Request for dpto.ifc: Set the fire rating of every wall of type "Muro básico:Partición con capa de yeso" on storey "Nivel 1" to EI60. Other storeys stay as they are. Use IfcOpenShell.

First a look at what the model holds.

```python
import ifcopenshell
import ifcopenshell.util.element

model = ifcopenshell.open("dpto.ifc")
print(model.schema)
storey = next(s for s in model.by_type("IfcBuildingStorey") if s.Name == "Nivel 1")
walls = [e for e in ifcopenshell.util.element.get_decomposition(storey) if e.is_a("IfcWall")]
seen = {}
for e in walls:
    element_type = ifcopenshell.util.element.get_type(e)
    key = (element_type.Name if element_type != e and element_type else None, ifcopenshell.util.element.get_pset(e, "Pset_WallCommon", "FireRating"))
    seen[key] = seen.get(key, 0) + 1
for (name, value), count in sorted(seen.items(), key=str):
    print(count, "x", name, "|", value)
```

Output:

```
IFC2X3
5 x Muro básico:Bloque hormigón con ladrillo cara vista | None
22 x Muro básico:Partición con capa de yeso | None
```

```python
import ifcopenshell
import ifcopenshell.api.pset
import ifcopenshell.util.element

model = ifcopenshell.open("dpto.ifc")

storey = next(s for s in model.by_type("IfcBuildingStorey") if s.Name == "Nivel 1")
walls = [e for e in ifcopenshell.util.element.get_decomposition(storey) if e.is_a("IfcWall")]

count = 0
for e in walls:
    element_type = ifcopenshell.util.element.get_type(e)
    if element_type in (None, e) or element_type.Name != "Muro básico:Partición con capa de yeso":
        continue
    # add_pset returns the element's existing set when there is one.
    pset = ifcopenshell.api.pset.add_pset(model, product=e, name="Pset_WallCommon")
    ifcopenshell.api.pset.edit_pset(model, pset=pset, properties={"FireRating": "EI60"})
    count += 1

print(count, "walls updated")

model.write("dpto_edited.ifc")
```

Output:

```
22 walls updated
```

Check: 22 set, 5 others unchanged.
